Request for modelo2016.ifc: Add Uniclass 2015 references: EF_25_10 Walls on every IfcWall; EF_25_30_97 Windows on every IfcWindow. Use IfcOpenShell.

First a look at what the model holds.

```python
import ifcopenshell

model = ifcopenshell.open("modelo2016.ifc")
print(model.schema)
print("classifications:", [c.Name for c in model.by_type("IfcClassification")])
for ifc_class in ("IfcDoor", "IfcRoof", "IfcStair", "IfcWall", "IfcWindow"):
    print(ifc_class, len(model.by_type(ifc_class)))
```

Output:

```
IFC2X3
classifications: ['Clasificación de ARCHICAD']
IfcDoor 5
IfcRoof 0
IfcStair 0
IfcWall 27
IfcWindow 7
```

```python
import ifcopenshell
import ifcopenshell.api.classification

model = ifcopenshell.open("modelo2016.ifc")

# IFC2X3 requires Source and Edition and has no link from the project to the system.
system = model.create_entity("IfcClassification", Source="NBS", Edition="2015", Name="Uniclass 2015")

codes = {
    "IfcWall": ("EF_25_10", "Walls"),
    "IfcWindow": ("EF_25_30_97", "Windows"),
}
for ifc_class, (code, name) in codes.items():
    products = model.by_type(ifc_class)
    ifcopenshell.api.classification.add_reference(
        model, products=products, classification=system, identification=code, name=name
    )
    print(code, len(products))

model.write("modelo2016_rev.ifc")
```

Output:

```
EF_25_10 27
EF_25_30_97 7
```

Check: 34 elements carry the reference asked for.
